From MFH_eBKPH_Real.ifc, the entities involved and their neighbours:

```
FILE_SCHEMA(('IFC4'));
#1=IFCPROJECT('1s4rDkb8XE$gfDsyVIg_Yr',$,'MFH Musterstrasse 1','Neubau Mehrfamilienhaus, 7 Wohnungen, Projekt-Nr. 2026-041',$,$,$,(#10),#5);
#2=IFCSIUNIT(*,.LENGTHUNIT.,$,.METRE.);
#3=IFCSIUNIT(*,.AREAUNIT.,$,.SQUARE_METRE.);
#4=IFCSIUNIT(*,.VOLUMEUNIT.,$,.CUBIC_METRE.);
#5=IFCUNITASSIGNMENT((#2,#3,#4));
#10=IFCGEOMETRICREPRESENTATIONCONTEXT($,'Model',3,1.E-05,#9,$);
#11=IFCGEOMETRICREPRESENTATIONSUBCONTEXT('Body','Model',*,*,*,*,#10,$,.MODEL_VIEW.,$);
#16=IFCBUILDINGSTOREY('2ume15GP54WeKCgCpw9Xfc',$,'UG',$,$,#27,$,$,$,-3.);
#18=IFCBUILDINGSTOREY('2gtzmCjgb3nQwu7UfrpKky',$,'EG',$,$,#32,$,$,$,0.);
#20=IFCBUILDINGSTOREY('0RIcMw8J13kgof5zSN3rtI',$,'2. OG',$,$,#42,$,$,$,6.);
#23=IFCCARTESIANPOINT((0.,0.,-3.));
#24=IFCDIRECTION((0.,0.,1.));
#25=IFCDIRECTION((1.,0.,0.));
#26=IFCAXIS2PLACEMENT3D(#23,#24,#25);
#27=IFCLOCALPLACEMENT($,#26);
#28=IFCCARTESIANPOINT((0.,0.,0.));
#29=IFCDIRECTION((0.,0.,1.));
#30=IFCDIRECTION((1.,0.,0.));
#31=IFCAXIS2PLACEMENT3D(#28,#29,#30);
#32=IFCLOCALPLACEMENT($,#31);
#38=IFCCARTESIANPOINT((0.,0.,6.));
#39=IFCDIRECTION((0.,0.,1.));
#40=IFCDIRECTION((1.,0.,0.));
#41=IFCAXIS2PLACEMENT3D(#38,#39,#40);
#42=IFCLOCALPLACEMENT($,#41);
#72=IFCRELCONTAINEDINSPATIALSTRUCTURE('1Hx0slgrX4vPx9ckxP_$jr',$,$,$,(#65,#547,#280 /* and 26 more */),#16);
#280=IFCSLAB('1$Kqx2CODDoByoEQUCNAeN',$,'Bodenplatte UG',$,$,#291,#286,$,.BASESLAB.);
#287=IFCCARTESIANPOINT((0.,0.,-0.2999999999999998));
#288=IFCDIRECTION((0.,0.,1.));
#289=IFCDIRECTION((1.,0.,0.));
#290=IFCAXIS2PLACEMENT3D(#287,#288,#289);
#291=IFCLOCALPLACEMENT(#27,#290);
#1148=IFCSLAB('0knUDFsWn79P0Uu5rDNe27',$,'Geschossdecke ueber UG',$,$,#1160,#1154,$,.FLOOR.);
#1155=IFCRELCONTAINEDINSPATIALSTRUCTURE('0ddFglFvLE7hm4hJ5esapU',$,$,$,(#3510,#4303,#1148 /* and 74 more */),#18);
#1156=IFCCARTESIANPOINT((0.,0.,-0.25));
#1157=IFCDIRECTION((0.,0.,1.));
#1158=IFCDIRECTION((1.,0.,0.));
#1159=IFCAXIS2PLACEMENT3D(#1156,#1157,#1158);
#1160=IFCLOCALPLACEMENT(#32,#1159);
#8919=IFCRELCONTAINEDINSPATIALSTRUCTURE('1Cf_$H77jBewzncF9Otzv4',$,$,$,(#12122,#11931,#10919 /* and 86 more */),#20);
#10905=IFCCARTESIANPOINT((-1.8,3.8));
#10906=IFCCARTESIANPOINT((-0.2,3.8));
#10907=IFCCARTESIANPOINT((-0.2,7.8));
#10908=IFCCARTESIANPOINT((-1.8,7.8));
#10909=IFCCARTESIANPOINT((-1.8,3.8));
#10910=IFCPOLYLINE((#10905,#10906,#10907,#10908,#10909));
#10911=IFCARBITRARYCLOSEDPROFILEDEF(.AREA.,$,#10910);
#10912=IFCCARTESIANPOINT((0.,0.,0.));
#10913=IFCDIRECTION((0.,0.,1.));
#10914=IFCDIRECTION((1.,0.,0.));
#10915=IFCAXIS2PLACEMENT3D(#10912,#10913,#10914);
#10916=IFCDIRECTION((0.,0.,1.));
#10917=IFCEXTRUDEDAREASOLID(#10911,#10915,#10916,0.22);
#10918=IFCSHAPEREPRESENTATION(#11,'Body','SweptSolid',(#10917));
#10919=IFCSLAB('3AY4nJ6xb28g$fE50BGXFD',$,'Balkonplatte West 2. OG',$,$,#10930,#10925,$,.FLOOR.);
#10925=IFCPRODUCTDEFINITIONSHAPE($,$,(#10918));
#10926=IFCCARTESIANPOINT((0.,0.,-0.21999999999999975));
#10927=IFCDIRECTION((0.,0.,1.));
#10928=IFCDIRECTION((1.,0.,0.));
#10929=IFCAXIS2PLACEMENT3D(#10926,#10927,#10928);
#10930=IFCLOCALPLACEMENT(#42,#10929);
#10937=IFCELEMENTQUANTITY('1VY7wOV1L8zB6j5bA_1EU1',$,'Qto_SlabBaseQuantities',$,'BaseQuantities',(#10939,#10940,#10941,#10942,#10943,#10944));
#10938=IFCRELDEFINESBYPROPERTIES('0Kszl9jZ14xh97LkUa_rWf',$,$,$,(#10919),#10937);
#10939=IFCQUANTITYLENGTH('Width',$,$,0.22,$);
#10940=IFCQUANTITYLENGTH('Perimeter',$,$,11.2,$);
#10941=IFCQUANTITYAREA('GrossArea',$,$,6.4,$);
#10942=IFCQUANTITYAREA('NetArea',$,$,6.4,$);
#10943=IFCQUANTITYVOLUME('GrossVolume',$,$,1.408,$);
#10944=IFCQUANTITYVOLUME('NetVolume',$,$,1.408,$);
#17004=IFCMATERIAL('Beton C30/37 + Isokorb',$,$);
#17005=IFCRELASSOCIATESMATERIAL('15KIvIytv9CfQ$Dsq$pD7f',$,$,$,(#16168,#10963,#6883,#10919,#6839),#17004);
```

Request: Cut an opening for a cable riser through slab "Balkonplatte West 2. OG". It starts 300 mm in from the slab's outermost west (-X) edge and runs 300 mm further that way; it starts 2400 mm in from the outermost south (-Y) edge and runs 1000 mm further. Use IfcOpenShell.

```python
import numpy as np
import ifcopenshell
import ifcopenshell.api.feature
import ifcopenshell.api.geometry
import ifcopenshell.api.pset
import ifcopenshell.api.root
import ifcopenshell.geom
import ifcopenshell.util.element
import ifcopenshell.util.placement
import ifcopenshell.util.representation
import ifcopenshell.util.shape
import ifcopenshell.util.unit

model = ifcopenshell.open("MFH_eBKPH_Real.ifc")
unit_scale = ifcopenshell.util.unit.calculate_unit_scale(model)
area_scale = ifcopenshell.util.unit.calculate_unit_scale(model, "AREAUNIT")
volume_scale = ifcopenshell.util.unit.calculate_unit_scale(model, "VOLUMEUNIT")
settings = ifcopenshell.geom.settings()


def volume(element):
    """Net volume in cubic metres, openings subtracted."""
    shape = ifcopenshell.geom.create_shape(settings, element)
    return ifcopenshell.util.shape.get_volume(shape.geometry)


slab = model.by_guid("3AY4nJ6xb28g$fE50BGXFD")
before = volume(slab)

# Extent in the slab's own axes, in metres. The edges named are its -X and -Y sides.
slab_shape = ifcopenshell.geom.create_shape(settings, slab)
vertices = ifcopenshell.util.shape.get_vertices(slab_shape.geometry)
x_min, y_min, bottom = vertices.min(axis=0)
top = vertices[:, 2].max()

opening = ifcopenshell.api.root.create_entity(model, ifc_class="IfcOpeningElement", name="Cable riser opening", predefined_type="OPENING")
context = ifcopenshell.util.representation.get_context(model, "Model", "Body", "MODEL_VIEW")
width, depth = 0.3, 1
outline = [(0.0, 0.0), (width, 0.0), (width, depth), (0.0, depth), (0.0, 0.0)]
# Overshoot both faces by 50 mm so the cut is clean.
shape = ifcopenshell.api.geometry.add_slab_representation(
    model, context=context, depth=top - bottom + 0.1, polyline=outline
)
ifcopenshell.api.geometry.assign_representation(model, product=opening, representation=shape)

matrix = ifcopenshell.util.placement.get_local_placement(slab.ObjectPlacement)
matrix[:, 3] = matrix @ np.append(np.array([x_min + 0.3, y_min + 2.4, bottom - 0.05]) / unit_scale, 1.0)
ifcopenshell.api.geometry.edit_object_placement(model, product=opening, matrix=matrix, is_si=False)
ifcopenshell.api.feature.add_feature(model, feature=opening, element=slab)

after = volume(slab)

# Update the slab's stored quantities.
qto = model.by_id(ifcopenshell.util.element.get_pset(slab, "Qto_SlabBaseQuantities", should_inherit=False)["id"])
ifcopenshell.api.pset.edit_qto(model, qto=qto, properties={
    "NetArea": after / (top - bottom) / area_scale,
    "NetVolume": after / volume_scale,
})

print(f"slab volume {before:.3f} -> {after:.3f} m3")

model.write("MFH_eBKPH_Real-out.ifc")
```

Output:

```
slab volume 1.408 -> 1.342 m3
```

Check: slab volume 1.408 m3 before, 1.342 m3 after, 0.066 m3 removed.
